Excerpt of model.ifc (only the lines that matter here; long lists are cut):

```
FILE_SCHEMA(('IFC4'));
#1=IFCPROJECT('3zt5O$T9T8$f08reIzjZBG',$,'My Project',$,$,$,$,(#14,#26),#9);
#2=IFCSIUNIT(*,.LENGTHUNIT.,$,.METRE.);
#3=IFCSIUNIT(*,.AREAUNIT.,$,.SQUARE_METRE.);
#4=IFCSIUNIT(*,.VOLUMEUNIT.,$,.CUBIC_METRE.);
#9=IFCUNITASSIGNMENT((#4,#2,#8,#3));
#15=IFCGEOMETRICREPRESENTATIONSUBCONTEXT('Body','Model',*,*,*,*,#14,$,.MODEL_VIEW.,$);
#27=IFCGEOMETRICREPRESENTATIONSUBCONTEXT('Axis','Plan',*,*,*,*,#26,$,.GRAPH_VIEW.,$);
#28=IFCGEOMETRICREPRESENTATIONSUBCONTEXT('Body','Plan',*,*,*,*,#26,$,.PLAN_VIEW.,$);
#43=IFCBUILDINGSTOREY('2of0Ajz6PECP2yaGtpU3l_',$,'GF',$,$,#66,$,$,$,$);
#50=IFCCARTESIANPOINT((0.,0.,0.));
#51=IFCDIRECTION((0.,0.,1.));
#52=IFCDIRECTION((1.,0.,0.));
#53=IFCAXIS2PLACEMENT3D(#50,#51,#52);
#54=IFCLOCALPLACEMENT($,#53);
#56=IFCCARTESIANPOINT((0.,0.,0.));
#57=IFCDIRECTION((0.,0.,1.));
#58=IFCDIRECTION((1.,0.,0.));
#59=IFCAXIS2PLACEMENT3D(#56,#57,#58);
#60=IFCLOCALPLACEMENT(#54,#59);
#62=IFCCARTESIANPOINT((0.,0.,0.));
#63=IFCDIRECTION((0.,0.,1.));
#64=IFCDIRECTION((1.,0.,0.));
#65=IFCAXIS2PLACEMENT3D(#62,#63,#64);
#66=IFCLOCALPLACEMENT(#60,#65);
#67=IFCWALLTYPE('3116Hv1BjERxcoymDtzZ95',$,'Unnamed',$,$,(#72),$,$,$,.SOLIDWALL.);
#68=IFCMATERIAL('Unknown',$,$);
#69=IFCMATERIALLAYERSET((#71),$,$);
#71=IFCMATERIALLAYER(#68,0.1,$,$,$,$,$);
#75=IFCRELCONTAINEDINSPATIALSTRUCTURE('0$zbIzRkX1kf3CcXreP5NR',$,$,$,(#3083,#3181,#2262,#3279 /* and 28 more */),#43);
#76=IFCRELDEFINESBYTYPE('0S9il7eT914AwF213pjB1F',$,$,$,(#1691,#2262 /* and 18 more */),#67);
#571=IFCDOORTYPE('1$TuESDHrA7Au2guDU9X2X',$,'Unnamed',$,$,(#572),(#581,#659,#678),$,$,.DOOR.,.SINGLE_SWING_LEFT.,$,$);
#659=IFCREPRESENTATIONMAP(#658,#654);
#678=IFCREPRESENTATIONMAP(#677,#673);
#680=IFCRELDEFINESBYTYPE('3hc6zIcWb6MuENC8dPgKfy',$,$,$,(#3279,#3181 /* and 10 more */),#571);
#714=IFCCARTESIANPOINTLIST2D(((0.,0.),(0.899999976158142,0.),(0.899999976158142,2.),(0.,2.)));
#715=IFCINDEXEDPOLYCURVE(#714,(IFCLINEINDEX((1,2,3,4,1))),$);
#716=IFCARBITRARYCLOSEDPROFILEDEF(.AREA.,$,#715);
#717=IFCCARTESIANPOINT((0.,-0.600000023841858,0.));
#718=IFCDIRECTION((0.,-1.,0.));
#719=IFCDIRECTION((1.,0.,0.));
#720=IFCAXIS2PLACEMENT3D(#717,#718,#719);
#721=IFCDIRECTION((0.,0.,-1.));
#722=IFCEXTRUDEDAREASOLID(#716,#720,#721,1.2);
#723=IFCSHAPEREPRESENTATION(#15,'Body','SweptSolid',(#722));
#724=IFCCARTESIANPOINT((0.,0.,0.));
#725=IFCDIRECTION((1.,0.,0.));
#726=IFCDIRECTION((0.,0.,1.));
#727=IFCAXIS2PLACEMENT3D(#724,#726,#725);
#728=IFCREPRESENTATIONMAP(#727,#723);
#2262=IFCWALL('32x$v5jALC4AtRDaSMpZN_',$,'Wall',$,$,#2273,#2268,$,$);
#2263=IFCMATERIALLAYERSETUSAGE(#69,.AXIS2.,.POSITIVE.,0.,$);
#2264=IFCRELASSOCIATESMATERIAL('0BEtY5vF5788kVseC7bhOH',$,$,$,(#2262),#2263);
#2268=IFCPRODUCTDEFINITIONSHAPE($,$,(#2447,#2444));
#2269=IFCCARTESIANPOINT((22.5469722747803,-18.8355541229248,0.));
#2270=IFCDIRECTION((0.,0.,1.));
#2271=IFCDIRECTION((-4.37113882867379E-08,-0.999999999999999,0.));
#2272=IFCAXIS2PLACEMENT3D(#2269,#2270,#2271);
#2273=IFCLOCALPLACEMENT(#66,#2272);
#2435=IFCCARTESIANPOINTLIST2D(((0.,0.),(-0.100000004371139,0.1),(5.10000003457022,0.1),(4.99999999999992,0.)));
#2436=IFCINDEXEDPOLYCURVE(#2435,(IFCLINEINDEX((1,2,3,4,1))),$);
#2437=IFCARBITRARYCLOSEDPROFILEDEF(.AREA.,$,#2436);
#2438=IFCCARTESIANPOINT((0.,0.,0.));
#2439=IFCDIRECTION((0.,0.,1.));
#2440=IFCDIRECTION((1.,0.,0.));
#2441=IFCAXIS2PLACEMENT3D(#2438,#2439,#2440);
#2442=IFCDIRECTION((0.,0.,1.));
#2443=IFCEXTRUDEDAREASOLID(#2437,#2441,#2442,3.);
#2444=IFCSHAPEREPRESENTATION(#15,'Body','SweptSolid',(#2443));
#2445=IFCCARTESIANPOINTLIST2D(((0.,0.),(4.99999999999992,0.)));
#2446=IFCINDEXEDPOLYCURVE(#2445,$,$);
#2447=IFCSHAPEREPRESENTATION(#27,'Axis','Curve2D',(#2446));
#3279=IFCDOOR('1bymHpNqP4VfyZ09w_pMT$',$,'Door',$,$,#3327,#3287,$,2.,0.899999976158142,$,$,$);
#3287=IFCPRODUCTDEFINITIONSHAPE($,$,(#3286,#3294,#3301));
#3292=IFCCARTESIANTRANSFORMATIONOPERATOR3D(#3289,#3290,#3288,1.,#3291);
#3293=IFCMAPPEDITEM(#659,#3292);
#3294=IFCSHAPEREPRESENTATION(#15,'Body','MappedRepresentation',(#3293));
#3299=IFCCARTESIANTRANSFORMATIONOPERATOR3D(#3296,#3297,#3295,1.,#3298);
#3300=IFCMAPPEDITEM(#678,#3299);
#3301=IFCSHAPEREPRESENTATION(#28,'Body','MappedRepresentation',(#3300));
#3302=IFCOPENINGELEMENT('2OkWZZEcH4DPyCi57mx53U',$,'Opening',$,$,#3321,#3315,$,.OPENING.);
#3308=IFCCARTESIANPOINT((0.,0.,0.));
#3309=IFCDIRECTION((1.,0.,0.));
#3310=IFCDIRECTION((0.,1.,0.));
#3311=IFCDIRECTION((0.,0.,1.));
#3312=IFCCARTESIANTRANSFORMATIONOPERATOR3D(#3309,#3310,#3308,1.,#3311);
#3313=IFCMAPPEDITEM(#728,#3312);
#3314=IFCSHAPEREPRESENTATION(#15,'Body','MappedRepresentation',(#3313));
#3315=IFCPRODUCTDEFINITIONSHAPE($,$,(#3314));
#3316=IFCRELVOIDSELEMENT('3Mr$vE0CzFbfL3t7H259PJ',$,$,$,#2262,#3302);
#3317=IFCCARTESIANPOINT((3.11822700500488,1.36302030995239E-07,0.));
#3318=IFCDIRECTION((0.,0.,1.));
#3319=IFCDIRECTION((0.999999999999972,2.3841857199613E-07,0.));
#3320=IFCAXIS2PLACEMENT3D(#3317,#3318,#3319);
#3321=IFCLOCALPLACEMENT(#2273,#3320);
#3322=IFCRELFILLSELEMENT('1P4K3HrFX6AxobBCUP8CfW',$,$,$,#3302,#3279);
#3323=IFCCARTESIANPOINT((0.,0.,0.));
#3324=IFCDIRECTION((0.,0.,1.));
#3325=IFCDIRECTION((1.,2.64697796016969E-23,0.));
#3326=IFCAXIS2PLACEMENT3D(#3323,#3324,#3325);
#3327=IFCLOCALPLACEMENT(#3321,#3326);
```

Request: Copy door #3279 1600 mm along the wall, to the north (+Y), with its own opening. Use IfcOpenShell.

```python
import ifcopenshell
import ifcopenshell.api.feature
import ifcopenshell.api.geometry
import ifcopenshell.api.root
import ifcopenshell.geom
import ifcopenshell.util.element
import ifcopenshell.util.placement
import ifcopenshell.util.shape

model = ifcopenshell.open("model.ifc")
settings = ifcopenshell.geom.settings()


def volume(element):
    """Net volume in cubic metres, openings subtracted."""
    shape = ifcopenshell.geom.create_shape(settings, element)
    return ifcopenshell.util.shape.get_volume(shape.geometry)


door = model.by_guid("1bymHpNqP4VfyZ09w_pMT$")
opening = door.FillsVoids[0].RelatingOpeningElement
wall = opening.VoidsElements[0].RelatingBuildingElement
before = volume(wall)
shift = ifcopenshell.util.placement.get_local_placement(wall.ObjectPlacement)[:3, 0] * -1.6

# copy_class copies the void relationship, type, container and properties, but no geometry.
new_opening = ifcopenshell.api.root.copy_class(model, product=opening)
new_opening.Representation = ifcopenshell.util.element.copy_deep(
    model, opening.Representation, exclude=["IfcGeometricRepresentationContext", "IfcRepresentationMap"]
)
new_door = ifcopenshell.api.root.copy_class(model, product=door)
new_door.Representation = ifcopenshell.util.element.copy_deep(
    model, door.Representation, exclude=["IfcGeometricRepresentationContext", "IfcRepresentationMap"]
)
ifcopenshell.api.feature.add_filling(model, opening=new_opening, element=new_door)

for old, new in ((opening, new_opening), (door, new_door)):
    matrix = ifcopenshell.util.placement.get_local_placement(old.ObjectPlacement)
    matrix[:3, 3] += shift
    ifcopenshell.api.geometry.edit_object_placement(model, product=new, matrix=matrix, is_si=False)

after = volume(wall)

print(f"wall volume {before:.3f} -> {after:.3f} m3")

model.write("model_v2.ifc")
```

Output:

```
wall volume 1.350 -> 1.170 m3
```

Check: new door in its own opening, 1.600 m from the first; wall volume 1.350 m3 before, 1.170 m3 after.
